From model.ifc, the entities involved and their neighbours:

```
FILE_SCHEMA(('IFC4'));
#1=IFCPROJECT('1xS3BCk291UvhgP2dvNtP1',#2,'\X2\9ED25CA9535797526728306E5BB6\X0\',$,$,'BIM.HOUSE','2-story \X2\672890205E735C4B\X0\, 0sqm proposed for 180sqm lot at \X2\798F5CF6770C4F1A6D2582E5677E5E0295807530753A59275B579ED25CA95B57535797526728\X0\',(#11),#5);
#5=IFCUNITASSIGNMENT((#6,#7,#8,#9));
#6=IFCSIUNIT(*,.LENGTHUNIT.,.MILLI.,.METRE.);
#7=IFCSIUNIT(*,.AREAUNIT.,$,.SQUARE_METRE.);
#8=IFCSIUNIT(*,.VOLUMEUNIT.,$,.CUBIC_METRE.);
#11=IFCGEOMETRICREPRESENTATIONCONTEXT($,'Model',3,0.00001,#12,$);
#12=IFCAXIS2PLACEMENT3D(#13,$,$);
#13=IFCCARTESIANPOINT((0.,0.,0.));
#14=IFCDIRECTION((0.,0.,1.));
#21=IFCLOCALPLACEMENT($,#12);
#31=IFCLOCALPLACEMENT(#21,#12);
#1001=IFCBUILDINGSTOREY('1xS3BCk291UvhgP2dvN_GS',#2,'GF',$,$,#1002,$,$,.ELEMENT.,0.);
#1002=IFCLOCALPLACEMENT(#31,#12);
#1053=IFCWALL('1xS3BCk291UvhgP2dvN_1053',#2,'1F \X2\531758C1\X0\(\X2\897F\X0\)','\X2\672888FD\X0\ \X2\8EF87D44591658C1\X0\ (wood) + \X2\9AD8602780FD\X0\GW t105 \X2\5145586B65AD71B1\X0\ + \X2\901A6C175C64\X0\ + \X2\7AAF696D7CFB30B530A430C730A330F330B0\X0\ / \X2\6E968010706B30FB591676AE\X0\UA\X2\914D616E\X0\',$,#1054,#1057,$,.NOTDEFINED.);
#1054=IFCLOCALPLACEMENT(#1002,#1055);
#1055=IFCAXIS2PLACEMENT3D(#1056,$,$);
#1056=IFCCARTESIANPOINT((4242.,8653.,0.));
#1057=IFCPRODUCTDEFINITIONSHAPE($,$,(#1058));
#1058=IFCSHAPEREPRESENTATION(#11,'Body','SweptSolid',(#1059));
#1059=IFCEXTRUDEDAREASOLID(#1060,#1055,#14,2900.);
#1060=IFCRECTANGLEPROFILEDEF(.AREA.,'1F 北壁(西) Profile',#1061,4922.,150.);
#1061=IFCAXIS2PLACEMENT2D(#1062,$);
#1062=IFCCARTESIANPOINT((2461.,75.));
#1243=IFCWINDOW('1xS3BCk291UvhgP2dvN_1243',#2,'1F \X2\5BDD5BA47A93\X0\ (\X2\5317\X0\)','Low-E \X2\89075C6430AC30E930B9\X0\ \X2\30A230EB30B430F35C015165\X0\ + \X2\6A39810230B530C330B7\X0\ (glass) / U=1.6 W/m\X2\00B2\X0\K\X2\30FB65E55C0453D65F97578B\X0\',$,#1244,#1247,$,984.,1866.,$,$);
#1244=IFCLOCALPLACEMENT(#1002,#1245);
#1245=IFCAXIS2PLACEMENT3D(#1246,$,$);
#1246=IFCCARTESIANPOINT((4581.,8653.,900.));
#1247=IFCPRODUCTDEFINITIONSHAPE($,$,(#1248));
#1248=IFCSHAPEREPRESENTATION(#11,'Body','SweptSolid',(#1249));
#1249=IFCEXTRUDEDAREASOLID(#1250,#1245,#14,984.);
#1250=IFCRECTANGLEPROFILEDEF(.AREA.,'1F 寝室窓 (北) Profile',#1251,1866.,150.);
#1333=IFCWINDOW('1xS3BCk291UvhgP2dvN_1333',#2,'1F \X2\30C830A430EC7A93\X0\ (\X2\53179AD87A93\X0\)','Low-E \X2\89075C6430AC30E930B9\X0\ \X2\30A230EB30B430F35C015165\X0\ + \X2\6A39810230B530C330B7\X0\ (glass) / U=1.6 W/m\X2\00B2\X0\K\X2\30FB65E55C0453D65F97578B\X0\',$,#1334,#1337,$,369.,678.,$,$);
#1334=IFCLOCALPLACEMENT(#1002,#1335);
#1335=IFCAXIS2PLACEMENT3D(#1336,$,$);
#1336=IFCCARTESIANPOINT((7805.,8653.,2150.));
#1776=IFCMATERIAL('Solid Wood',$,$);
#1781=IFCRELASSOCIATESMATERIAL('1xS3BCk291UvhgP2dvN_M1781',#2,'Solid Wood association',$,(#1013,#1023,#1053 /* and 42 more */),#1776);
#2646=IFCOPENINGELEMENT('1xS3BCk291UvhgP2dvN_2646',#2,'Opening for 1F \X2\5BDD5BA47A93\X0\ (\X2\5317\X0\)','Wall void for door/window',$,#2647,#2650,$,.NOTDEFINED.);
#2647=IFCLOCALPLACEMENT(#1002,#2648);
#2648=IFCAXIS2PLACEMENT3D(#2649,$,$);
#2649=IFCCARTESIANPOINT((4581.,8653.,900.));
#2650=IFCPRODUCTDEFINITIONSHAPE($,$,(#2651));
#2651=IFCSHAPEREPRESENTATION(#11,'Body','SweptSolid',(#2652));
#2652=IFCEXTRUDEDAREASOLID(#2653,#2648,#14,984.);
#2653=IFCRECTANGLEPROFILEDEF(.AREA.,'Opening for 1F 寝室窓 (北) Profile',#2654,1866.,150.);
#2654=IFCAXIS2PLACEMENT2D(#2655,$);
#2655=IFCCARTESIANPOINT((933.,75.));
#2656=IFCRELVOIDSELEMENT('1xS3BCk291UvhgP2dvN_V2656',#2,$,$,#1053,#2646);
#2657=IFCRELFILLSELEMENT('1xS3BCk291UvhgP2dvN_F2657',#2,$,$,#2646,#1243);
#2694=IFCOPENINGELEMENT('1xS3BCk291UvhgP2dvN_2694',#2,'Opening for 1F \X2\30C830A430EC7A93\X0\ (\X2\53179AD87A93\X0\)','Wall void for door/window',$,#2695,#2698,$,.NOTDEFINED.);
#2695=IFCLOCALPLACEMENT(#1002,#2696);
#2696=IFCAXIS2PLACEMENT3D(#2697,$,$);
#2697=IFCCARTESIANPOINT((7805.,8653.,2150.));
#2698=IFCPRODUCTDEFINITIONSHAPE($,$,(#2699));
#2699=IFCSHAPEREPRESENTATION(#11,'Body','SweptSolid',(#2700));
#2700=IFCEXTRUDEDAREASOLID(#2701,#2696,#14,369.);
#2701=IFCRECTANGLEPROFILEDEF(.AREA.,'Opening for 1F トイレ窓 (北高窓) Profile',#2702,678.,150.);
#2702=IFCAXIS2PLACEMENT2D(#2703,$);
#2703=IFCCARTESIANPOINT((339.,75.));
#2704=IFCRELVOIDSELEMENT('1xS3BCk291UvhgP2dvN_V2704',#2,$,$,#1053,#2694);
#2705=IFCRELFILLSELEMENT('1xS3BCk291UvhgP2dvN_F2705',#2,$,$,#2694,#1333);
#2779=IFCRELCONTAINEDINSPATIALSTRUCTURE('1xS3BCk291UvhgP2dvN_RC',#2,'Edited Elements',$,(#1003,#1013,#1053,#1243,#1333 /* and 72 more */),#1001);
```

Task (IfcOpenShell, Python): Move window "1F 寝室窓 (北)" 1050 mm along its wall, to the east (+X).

```python
import ifcopenshell
import ifcopenshell.api.geometry
import ifcopenshell.util.placement
import ifcopenshell.util.unit

model = ifcopenshell.open("model.ifc")
unit_scale = ifcopenshell.util.unit.calculate_unit_scale(model)

window = model.by_guid("1xS3BCk291UvhgP2dvN_1243")
opening = window.FillsVoids[0].RelatingOpeningElement
wall = opening.VoidsElements[0].RelatingBuildingElement

wall_matrix = ifcopenshell.util.placement.get_local_placement(wall.ObjectPlacement)
shift = wall_matrix[:3, 0] * 1.05 / unit_scale
before = ifcopenshell.util.placement.get_local_placement(window.ObjectPlacement)[:3, 3].copy()

# The window is not placed relative to its opening, so move both.
for product in (opening, window):
    matrix = ifcopenshell.util.placement.get_local_placement(product.ObjectPlacement)
    matrix[:3, 3] += shift
    ifcopenshell.api.geometry.edit_object_placement(model, product=product, matrix=matrix, is_si=False)

after = ifcopenshell.util.placement.get_local_placement(window.ObjectPlacement)[:3, 3]
print("window moved by", (after - before).round(3) + 0.0)

model.write("model_updated.ifc")
```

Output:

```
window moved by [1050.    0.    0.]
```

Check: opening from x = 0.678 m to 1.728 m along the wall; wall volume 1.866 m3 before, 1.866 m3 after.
